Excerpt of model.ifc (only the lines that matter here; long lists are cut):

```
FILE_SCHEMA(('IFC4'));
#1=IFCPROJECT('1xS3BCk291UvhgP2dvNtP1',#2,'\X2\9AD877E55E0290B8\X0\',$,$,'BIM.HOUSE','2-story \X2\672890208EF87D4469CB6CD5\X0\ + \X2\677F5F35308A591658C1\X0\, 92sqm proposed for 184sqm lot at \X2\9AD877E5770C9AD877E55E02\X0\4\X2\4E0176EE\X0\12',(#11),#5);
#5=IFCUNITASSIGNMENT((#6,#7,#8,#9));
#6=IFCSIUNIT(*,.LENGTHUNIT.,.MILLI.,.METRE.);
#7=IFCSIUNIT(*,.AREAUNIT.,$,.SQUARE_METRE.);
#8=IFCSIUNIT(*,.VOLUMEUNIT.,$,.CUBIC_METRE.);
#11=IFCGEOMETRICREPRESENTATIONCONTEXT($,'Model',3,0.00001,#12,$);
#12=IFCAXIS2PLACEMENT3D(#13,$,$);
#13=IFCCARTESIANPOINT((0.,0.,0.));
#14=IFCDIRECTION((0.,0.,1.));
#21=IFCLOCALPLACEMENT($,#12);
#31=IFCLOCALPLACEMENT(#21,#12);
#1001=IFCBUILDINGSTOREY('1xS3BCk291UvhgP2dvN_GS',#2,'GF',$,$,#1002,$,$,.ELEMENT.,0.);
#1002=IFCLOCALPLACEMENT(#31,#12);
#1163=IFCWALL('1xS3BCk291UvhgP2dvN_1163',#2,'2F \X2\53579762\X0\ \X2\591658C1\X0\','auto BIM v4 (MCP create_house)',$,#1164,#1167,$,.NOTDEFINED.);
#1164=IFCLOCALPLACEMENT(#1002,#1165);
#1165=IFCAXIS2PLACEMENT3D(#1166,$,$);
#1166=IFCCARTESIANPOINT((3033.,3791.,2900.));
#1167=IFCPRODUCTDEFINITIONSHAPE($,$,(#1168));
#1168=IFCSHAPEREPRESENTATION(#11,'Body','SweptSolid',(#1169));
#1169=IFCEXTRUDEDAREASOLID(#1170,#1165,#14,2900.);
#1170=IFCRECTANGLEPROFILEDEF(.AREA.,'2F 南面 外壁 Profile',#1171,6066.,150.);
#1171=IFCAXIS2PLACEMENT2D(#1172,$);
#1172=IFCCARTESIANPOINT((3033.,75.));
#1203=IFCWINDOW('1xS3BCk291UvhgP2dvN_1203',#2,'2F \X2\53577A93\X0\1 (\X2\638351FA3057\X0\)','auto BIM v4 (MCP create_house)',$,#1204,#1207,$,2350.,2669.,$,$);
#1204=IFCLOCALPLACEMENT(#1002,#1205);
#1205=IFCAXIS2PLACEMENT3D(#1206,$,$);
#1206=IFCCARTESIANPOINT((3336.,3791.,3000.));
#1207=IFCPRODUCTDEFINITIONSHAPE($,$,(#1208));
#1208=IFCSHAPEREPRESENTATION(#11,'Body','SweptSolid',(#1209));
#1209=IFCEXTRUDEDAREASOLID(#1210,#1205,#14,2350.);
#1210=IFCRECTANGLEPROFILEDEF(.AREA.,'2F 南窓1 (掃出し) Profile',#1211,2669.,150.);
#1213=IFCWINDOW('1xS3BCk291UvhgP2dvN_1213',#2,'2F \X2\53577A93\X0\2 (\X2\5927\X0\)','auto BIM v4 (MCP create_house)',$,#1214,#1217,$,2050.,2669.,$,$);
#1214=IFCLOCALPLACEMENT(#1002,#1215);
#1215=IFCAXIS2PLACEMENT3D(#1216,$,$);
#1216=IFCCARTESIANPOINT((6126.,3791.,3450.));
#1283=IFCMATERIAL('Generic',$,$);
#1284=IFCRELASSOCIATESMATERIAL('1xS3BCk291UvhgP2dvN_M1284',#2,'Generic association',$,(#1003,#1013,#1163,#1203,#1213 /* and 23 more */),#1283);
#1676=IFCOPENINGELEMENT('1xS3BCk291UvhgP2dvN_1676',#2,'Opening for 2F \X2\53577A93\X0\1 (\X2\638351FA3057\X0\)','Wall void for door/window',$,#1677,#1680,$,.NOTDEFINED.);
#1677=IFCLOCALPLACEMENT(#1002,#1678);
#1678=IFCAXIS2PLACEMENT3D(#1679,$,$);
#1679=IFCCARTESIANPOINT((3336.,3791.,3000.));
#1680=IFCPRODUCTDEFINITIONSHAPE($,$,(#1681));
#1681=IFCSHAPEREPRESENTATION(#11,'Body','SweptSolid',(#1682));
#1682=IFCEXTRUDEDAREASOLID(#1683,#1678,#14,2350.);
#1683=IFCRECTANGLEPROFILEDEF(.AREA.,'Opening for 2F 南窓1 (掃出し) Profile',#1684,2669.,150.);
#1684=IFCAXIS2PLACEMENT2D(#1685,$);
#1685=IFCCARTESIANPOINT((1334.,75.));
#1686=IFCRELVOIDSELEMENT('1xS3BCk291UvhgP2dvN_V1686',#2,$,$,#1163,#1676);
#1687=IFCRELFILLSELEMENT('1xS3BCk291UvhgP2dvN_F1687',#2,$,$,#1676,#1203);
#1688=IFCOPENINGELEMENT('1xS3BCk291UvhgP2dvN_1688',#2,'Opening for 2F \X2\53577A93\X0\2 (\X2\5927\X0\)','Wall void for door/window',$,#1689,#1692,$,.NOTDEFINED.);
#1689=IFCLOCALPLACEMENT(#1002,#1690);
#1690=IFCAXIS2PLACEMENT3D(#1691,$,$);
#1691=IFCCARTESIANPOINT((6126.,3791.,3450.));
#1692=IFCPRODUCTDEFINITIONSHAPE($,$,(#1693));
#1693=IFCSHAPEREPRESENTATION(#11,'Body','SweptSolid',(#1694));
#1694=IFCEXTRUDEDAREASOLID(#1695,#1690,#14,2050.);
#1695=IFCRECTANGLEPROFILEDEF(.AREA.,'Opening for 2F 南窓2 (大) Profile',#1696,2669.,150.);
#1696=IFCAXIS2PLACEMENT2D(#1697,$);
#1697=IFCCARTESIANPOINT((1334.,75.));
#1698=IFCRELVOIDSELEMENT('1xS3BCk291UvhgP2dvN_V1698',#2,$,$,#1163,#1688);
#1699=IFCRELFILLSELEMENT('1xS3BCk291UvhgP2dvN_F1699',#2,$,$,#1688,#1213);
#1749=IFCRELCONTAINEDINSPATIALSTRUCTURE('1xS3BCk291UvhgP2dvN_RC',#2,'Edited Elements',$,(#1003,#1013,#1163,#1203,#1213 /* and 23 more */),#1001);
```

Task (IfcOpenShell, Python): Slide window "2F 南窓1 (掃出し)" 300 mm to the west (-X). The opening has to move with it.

```python
import ifcopenshell
import ifcopenshell.api.geometry
import ifcopenshell.util.placement

model = ifcopenshell.open("model.ifc")

window = model.by_guid("1xS3BCk291UvhgP2dvN_1203")
opening = window.FillsVoids[0].RelatingOpeningElement
wall = opening.VoidsElements[0].RelatingBuildingElement

wall_matrix = ifcopenshell.util.placement.get_local_placement(wall.ObjectPlacement)
shift = wall_matrix[:3, 0] * -300.0
before = ifcopenshell.util.placement.get_local_placement(window.ObjectPlacement)[:3, 3].copy()

# The window is not placed relative to its opening, so move both.
for product in (opening, window):
    matrix = ifcopenshell.util.placement.get_local_placement(product.ObjectPlacement)
    matrix[:3, 3] += shift
    ifcopenshell.api.geometry.edit_object_placement(model, product=product, matrix=matrix, is_si=False)

after = ifcopenshell.util.placement.get_local_placement(window.ObjectPlacement)[:3, 3]
print("window moved by", (after - before).round(3) + 0.0)

model.write("model_edited.ifc")
```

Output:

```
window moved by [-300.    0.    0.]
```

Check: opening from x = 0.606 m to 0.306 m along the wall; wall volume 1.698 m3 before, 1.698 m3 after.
